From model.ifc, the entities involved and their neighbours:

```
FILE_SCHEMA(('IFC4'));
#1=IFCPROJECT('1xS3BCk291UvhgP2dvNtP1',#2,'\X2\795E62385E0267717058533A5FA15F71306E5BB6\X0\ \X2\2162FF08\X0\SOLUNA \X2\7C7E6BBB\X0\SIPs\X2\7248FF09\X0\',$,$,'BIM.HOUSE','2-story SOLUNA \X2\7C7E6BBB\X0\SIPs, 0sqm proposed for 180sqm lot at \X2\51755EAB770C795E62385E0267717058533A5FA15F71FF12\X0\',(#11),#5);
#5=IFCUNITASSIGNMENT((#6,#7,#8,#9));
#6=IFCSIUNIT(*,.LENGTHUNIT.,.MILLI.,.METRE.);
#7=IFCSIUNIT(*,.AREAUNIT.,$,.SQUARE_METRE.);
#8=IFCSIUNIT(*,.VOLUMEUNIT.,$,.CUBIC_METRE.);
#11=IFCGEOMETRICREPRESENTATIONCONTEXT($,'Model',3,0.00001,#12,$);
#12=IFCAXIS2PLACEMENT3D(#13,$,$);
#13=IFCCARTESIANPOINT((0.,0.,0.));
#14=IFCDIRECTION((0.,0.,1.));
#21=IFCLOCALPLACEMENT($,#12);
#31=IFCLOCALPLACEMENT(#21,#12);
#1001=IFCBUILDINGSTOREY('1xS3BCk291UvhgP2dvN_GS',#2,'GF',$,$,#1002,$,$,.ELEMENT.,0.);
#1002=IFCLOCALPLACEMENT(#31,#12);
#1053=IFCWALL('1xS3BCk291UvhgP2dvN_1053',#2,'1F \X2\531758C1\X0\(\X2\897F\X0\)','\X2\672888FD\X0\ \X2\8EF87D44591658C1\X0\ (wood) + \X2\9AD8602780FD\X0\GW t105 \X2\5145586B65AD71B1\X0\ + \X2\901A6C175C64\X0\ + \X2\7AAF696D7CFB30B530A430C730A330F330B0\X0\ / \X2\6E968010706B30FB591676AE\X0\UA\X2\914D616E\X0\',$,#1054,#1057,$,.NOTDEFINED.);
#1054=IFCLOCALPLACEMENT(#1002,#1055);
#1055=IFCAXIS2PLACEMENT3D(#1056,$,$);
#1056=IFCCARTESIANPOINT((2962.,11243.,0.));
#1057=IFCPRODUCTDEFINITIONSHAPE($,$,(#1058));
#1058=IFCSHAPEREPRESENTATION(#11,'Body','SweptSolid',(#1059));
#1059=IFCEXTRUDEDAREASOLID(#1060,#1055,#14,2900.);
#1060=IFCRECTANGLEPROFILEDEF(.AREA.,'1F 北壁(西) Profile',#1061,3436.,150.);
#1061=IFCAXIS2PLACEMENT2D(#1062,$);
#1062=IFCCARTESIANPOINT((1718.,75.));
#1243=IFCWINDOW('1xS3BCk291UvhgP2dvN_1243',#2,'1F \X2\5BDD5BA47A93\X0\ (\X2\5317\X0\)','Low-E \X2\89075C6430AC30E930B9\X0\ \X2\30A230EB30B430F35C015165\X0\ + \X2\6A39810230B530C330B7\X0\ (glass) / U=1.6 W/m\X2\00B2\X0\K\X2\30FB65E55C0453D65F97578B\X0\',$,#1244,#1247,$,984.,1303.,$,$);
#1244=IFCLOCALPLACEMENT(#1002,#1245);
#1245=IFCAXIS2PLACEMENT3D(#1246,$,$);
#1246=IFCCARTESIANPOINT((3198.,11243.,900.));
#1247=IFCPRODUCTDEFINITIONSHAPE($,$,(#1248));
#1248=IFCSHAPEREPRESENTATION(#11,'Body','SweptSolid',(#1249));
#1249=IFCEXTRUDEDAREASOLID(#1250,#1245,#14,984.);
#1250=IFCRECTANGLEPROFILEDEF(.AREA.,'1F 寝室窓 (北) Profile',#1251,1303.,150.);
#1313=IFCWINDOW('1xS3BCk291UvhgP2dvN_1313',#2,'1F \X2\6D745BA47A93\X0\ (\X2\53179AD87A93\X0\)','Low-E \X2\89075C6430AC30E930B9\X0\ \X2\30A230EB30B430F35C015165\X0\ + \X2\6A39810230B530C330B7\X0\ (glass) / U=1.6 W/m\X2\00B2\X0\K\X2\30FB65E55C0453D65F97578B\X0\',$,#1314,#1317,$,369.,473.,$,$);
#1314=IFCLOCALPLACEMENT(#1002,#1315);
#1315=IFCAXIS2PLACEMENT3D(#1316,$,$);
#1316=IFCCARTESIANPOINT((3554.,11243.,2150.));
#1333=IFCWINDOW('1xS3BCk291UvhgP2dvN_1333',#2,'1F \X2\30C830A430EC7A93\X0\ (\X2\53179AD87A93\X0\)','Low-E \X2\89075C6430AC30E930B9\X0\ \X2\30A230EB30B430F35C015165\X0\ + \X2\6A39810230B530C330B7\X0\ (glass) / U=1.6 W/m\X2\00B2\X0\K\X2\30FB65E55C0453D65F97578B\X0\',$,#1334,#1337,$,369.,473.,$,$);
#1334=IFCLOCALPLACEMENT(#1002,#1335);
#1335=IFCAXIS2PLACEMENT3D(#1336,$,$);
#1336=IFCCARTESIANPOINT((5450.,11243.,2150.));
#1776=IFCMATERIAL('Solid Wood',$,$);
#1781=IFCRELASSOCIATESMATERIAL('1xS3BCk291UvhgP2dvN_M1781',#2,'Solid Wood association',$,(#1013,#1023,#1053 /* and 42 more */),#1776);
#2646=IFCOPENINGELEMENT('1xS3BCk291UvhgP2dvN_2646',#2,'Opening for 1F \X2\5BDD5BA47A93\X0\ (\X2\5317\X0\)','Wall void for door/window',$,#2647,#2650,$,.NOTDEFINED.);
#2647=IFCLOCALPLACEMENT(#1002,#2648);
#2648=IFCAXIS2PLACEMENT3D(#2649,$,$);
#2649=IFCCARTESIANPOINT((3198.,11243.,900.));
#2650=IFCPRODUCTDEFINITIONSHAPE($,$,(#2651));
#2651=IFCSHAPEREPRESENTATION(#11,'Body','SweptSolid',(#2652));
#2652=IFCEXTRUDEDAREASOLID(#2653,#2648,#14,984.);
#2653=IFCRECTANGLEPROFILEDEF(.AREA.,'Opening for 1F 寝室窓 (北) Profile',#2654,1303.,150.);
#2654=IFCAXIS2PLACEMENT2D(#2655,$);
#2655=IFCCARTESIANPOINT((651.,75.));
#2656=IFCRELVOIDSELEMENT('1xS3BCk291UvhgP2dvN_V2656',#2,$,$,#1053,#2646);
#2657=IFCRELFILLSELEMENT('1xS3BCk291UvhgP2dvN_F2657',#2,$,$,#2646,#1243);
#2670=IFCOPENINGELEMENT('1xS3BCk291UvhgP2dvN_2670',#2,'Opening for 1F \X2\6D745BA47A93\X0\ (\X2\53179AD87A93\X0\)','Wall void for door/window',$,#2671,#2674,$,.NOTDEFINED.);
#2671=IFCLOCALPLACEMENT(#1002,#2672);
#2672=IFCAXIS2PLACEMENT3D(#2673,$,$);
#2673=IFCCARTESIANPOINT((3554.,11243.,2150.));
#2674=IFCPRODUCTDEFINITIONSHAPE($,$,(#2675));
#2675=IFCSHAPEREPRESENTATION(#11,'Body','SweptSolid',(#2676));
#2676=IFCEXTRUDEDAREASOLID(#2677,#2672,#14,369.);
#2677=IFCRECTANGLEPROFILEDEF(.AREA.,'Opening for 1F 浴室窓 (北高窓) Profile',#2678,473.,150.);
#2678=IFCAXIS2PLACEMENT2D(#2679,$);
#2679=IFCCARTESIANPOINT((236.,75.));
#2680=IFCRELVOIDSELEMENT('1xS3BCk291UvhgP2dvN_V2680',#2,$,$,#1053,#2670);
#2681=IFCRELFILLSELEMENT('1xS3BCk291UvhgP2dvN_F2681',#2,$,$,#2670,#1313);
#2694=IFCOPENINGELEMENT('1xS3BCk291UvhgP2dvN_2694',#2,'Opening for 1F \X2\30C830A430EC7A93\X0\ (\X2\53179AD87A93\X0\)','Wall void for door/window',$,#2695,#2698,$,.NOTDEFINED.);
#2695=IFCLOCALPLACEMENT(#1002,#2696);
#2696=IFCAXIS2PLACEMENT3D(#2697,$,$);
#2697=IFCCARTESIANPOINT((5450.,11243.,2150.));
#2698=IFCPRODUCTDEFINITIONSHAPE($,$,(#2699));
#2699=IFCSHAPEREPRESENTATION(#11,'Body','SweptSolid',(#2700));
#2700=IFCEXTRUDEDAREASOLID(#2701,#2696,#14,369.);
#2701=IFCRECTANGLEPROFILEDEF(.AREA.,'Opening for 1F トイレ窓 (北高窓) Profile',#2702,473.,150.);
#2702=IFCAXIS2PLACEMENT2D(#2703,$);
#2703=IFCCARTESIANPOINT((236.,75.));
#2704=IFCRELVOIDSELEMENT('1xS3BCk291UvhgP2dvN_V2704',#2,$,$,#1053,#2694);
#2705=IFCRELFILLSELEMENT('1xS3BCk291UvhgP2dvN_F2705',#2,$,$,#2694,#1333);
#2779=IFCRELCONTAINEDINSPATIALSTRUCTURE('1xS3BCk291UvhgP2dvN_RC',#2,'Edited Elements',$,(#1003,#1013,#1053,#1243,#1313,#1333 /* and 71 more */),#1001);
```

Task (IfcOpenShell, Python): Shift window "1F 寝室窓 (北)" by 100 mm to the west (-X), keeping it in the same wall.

```python
import ifcopenshell
import ifcopenshell.api.geometry
import ifcopenshell.util.placement
import ifcopenshell.util.unit

model = ifcopenshell.open("model.ifc")
unit_scale = ifcopenshell.util.unit.calculate_unit_scale(model)

window = model.by_guid("1xS3BCk291UvhgP2dvN_1243")
opening = window.FillsVoids[0].RelatingOpeningElement
wall = opening.VoidsElements[0].RelatingBuildingElement

wall_matrix = ifcopenshell.util.placement.get_local_placement(wall.ObjectPlacement)
shift = wall_matrix[:3, 0] * -0.1 / unit_scale
before = ifcopenshell.util.placement.get_local_placement(window.ObjectPlacement)[:3, 3].copy()

# The window is not placed relative to its opening, so move both.
for product in (opening, window):
    matrix = ifcopenshell.util.placement.get_local_placement(product.ObjectPlacement)
    matrix[:3, 3] += shift
    ifcopenshell.api.geometry.edit_object_placement(model, product=product, matrix=matrix, is_si=False)

after = ifcopenshell.util.placement.get_local_placement(window.ObjectPlacement)[:3, 3]
print("window moved by", (after - before).round(3) + 0.0)

model.write("model_updated.ifc")
```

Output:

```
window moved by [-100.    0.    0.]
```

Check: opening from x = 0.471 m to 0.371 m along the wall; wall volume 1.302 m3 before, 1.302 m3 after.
